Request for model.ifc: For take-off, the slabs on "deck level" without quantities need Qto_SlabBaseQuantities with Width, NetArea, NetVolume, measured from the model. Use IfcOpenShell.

First a look at what the model holds.

```python
import ifcopenshell
import ifcopenshell.util.element
import ifcopenshell.util.unit

model = ifcopenshell.open("model.ifc")
print(model.schema)
for unit_type in ("LENGTHUNIT", "AREAUNIT", "VOLUMEUNIT"):
    print(unit_type, ifcopenshell.util.unit.calculate_unit_scale(model, unit_type))
storey = next(s for s in model.by_type("IfcBuildingStorey") if s.Name == "deck level")
slabs = [e for e in ifcopenshell.util.element.get_decomposition(storey) if e.is_a("IfcSlab")]
for e in sorted(slabs, key=lambda e: e.id()):
    print(e.id(), e.is_a(), e.Name, list(ifcopenshell.util.element.get_psets(e, qtos_only=True)), sep=" | ")
```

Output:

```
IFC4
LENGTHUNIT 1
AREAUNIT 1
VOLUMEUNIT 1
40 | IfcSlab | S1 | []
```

```python
import ifcopenshell
import ifcopenshell.api.pset
import ifcopenshell.geom
import ifcopenshell.util.element
import ifcopenshell.util.shape
import ifcopenshell.util.unit

model = ifcopenshell.open("model.ifc")
unit_scale = ifcopenshell.util.unit.calculate_unit_scale(model)
area_scale = ifcopenshell.util.unit.calculate_unit_scale(model, "AREAUNIT")
volume_scale = ifcopenshell.util.unit.calculate_unit_scale(model, "VOLUMEUNIT")
settings = ifcopenshell.geom.settings()

storey = next(s for s in model.by_type("IfcBuildingStorey") if s.Name == "deck level")
slabs = [e for e in ifcopenshell.util.element.get_decomposition(storey) if e.is_a("IfcSlab")]

for e in sorted(slabs, key=lambda e: e.id()):
    if ifcopenshell.util.element.get_psets(e, qtos_only=True, should_inherit=False):
        continue
    # Geometry comes back in metres, in the element's own axes.
    shape = ifcopenshell.geom.create_shape(settings, e)
    values = {
        "Width": ifcopenshell.util.shape.get_z(shape.geometry) / unit_scale,
        "NetArea": ifcopenshell.util.shape.get_footprint_area(shape.geometry) / area_scale,
        "NetVolume": ifcopenshell.util.shape.get_volume(shape.geometry) / volume_scale,
    }
    qto = ifcopenshell.api.pset.add_qto(model, product=e, name="Qto_SlabBaseQuantities")
    ifcopenshell.api.pset.edit_qto(model, qto=qto, properties=values)
    print(e.id(), {k: round(v, 3) for k, v in values.items()})

model.write("model_updated.ifc")
```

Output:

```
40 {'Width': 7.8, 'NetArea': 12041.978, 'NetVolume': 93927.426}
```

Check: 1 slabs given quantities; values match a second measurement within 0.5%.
